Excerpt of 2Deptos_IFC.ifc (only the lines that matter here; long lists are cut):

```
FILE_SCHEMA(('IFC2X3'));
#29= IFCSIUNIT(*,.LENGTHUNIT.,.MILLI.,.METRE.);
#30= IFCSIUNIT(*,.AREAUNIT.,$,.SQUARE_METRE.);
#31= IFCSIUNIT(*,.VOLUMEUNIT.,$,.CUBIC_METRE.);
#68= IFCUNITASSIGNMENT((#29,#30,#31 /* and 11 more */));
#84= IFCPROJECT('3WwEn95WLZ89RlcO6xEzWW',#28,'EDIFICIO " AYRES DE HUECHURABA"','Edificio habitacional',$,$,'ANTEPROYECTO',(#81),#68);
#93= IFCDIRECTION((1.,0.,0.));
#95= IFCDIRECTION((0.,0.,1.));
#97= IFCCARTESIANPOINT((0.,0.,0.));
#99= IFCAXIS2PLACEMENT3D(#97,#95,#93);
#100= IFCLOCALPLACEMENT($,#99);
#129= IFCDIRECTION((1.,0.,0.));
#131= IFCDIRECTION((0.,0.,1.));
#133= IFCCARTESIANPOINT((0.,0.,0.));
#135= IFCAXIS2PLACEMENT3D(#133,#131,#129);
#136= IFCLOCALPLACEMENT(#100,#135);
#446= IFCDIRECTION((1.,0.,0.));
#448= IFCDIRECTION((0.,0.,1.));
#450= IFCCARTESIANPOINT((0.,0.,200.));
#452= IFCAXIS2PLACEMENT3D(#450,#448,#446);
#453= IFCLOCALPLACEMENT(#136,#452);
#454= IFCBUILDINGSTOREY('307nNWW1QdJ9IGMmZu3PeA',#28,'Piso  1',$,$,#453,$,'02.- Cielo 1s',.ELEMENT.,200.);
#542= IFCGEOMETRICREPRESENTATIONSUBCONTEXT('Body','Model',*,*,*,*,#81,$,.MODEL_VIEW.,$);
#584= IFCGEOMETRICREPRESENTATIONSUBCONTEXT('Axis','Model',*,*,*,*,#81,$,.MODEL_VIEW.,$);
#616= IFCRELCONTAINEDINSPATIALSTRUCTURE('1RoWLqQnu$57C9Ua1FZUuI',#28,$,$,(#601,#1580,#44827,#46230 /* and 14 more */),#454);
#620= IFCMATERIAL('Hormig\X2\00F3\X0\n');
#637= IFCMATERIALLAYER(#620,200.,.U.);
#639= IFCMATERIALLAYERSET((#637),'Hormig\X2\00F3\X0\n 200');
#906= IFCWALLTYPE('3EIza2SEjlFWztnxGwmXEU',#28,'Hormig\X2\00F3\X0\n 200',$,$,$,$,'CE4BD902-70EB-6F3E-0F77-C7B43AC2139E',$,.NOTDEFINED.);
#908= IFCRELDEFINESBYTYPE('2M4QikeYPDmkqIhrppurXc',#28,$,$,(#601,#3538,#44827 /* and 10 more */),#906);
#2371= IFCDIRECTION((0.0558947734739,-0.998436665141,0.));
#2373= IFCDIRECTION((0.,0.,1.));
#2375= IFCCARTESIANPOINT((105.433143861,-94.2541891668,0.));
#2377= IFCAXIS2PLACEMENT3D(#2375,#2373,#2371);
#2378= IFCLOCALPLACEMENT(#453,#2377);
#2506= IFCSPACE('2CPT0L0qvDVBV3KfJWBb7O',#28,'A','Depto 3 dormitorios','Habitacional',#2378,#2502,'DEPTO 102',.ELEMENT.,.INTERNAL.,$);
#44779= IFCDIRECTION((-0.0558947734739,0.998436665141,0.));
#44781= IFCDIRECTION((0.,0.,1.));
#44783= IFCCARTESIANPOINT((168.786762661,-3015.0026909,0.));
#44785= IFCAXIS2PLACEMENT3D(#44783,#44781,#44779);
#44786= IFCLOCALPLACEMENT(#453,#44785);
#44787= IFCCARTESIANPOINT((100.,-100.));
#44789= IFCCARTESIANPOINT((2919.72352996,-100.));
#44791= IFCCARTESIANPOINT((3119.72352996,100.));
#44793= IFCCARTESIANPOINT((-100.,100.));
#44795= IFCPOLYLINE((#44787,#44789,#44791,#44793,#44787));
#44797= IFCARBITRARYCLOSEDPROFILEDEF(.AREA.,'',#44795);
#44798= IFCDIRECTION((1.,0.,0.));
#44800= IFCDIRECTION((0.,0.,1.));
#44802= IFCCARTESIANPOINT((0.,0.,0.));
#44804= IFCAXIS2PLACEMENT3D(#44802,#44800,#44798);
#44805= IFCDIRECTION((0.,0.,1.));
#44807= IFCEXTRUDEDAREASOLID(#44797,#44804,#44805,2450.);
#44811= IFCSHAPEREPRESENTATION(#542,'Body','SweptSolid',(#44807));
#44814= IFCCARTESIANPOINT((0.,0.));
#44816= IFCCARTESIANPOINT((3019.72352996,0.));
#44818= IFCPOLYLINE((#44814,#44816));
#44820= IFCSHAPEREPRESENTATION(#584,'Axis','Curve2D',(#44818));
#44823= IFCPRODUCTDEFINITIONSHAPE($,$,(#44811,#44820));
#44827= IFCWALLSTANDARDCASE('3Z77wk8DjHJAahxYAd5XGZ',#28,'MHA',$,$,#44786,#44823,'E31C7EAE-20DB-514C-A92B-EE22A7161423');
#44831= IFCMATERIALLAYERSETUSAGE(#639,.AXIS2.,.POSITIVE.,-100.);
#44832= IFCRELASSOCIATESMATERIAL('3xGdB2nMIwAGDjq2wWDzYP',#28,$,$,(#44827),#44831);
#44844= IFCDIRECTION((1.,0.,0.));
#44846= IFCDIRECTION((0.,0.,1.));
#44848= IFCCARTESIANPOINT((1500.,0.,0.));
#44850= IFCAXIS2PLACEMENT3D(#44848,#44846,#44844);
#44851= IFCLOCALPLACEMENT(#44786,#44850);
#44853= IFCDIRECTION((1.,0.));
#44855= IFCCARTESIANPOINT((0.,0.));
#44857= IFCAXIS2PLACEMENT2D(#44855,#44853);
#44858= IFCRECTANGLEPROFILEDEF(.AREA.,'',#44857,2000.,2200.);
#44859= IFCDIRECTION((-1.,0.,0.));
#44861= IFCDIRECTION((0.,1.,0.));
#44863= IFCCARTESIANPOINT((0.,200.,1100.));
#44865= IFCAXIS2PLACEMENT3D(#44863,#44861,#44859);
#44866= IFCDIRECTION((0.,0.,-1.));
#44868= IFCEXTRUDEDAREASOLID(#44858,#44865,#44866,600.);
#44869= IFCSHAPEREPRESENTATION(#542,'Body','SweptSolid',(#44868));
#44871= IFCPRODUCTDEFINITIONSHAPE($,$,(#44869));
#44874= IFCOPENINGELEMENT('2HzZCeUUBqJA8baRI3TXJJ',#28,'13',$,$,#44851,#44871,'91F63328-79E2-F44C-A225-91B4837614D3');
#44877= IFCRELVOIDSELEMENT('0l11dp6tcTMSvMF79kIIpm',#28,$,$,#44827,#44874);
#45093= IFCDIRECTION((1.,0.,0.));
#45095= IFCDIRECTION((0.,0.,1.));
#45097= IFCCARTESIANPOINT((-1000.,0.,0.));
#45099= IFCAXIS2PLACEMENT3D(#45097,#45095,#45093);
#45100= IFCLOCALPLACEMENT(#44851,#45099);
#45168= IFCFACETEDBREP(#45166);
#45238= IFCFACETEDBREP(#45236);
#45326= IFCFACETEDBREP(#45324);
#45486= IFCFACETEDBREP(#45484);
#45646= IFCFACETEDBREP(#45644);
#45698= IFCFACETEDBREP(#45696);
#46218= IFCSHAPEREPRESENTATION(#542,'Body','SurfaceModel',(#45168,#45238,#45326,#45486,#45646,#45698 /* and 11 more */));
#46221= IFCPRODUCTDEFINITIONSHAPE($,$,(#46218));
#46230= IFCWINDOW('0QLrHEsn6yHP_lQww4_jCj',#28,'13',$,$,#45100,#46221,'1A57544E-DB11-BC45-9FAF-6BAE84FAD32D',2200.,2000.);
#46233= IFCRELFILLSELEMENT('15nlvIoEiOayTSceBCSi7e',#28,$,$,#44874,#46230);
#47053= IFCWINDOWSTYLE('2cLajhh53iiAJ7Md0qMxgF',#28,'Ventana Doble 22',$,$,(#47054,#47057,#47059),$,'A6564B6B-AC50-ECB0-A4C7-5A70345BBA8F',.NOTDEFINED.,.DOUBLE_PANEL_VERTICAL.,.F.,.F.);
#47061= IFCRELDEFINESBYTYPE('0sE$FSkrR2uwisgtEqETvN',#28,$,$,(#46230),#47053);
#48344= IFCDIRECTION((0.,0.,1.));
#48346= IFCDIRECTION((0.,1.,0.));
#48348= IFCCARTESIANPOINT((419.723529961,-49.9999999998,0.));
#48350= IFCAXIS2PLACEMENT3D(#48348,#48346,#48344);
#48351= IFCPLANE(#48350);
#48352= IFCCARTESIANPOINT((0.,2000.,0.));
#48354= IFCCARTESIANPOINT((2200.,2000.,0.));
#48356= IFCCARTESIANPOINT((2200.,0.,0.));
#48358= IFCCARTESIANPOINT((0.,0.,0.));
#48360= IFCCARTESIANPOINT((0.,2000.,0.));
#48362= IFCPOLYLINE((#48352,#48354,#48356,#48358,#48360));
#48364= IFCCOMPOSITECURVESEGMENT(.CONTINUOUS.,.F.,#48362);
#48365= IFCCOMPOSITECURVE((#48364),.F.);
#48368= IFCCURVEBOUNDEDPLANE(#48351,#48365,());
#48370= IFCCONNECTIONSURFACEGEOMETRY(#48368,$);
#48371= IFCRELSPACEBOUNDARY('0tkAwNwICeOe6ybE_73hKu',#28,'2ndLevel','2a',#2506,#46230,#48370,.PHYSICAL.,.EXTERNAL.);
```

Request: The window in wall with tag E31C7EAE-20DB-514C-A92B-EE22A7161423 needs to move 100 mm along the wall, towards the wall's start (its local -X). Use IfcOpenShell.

```python
import numpy as np
import ifcopenshell
import ifcopenshell.api.geometry
import ifcopenshell.util.placement
import ifcopenshell.util.unit

model = ifcopenshell.open("2Deptos_IFC.ifc")
unit_scale = ifcopenshell.util.unit.calculate_unit_scale(model)

window = model.by_guid("0QLrHEsn6yHP_lQww4_jCj")
opening = window.FillsVoids[0].RelatingOpeningElement
wall = opening.VoidsElements[0].RelatingBuildingElement

wall_matrix = ifcopenshell.util.placement.get_local_placement(wall.ObjectPlacement)
shift = wall_matrix[:3, 0] * -0.1 / unit_scale
before = ifcopenshell.util.placement.get_local_placement(window.ObjectPlacement)[:3, 3].copy()

# The window is placed relative to its opening, so it follows when the opening moves.
matrix = ifcopenshell.util.placement.get_local_placement(opening.ObjectPlacement)
matrix[:3, 3] += shift
ifcopenshell.api.geometry.edit_object_placement(
    model, product=opening, matrix=matrix, is_si=False, should_transform_children=True
)

# Space boundary surfaces are stored in each space's coordinates; move them too.
for rel in window.ProvidesBoundaries:
    if not rel.ConnectionGeometry:
        continue
    surface = rel.ConnectionGeometry.SurfaceOnRelatingElement.BasisSurface
    space_matrix = ifcopenshell.util.placement.get_local_placement(rel.RelatingSpace.ObjectPlacement)
    point = np.array(surface.Position.Location.Coordinates) + space_matrix[:3, :3].T @ shift
    surface.Position = model.createIfcAxis2Placement3D(
        model.createIfcCartesianPoint(point.tolist()), surface.Position.Axis, surface.Position.RefDirection
    )

after = ifcopenshell.util.placement.get_local_placement(window.ObjectPlacement)[:3, 3]
print("window moved by", (after - before).round(3) + 0.0)

model.write("2Deptos_IFC_rev.ifc")
```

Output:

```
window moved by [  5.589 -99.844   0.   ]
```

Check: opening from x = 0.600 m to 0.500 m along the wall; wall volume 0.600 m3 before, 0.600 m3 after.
